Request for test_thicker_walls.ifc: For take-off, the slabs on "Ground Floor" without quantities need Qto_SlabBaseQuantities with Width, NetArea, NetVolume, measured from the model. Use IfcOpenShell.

First a look at what the model holds.

```python
import ifcopenshell
import ifcopenshell.util.element
import ifcopenshell.util.unit

model = ifcopenshell.open("test_thicker_walls.ifc")
print(model.schema)
for unit_type in ("LENGTHUNIT", "AREAUNIT", "VOLUMEUNIT"):
    print(unit_type, ifcopenshell.util.unit.calculate_unit_scale(model, unit_type))
storey = next(s for s in model.by_type("IfcBuildingStorey") if s.Name == "Ground Floor")
slabs = [e for e in ifcopenshell.util.element.get_decomposition(storey) if e.is_a("IfcSlab")]
for e in sorted(slabs, key=lambda e: e.id()):
    print(e.id(), e.is_a(), e.Name, list(ifcopenshell.util.element.get_psets(e, qtos_only=True)), sep=" | ")
```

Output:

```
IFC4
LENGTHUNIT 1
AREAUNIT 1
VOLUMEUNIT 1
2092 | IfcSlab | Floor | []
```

```python
import ifcopenshell
import ifcopenshell.api.pset
import ifcopenshell.geom
import ifcopenshell.util.element
import ifcopenshell.util.shape
import ifcopenshell.util.unit

model = ifcopenshell.open("test_thicker_walls.ifc")
unit_scale = ifcopenshell.util.unit.calculate_unit_scale(model)
area_scale = ifcopenshell.util.unit.calculate_unit_scale(model, "AREAUNIT")
volume_scale = ifcopenshell.util.unit.calculate_unit_scale(model, "VOLUMEUNIT")
settings = ifcopenshell.geom.settings()

storey = next(s for s in model.by_type("IfcBuildingStorey") if s.Name == "Ground Floor")
slabs = [e for e in ifcopenshell.util.element.get_decomposition(storey) if e.is_a("IfcSlab")]

for e in sorted(slabs, key=lambda e: e.id()):
    if ifcopenshell.util.element.get_psets(e, qtos_only=True, should_inherit=False):
        continue
    # Geometry comes back in metres, in the element's own axes.
    shape = ifcopenshell.geom.create_shape(settings, e)
    values = {
        "Width": ifcopenshell.util.shape.get_z(shape.geometry) / unit_scale,
        "NetArea": ifcopenshell.util.shape.get_footprint_area(shape.geometry) / area_scale,
        "NetVolume": ifcopenshell.util.shape.get_volume(shape.geometry) / volume_scale,
    }
    qto = ifcopenshell.api.pset.add_qto(model, product=e, name="Qto_SlabBaseQuantities")
    ifcopenshell.api.pset.edit_qto(model, qto=qto, properties=values)
    print(e.id(), {k: round(v, 3) for k, v in values.items()})

model.write("test_thicker_walls_v2.ifc")
```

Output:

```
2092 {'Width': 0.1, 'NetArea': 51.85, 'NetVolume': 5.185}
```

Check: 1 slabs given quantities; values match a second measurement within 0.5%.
